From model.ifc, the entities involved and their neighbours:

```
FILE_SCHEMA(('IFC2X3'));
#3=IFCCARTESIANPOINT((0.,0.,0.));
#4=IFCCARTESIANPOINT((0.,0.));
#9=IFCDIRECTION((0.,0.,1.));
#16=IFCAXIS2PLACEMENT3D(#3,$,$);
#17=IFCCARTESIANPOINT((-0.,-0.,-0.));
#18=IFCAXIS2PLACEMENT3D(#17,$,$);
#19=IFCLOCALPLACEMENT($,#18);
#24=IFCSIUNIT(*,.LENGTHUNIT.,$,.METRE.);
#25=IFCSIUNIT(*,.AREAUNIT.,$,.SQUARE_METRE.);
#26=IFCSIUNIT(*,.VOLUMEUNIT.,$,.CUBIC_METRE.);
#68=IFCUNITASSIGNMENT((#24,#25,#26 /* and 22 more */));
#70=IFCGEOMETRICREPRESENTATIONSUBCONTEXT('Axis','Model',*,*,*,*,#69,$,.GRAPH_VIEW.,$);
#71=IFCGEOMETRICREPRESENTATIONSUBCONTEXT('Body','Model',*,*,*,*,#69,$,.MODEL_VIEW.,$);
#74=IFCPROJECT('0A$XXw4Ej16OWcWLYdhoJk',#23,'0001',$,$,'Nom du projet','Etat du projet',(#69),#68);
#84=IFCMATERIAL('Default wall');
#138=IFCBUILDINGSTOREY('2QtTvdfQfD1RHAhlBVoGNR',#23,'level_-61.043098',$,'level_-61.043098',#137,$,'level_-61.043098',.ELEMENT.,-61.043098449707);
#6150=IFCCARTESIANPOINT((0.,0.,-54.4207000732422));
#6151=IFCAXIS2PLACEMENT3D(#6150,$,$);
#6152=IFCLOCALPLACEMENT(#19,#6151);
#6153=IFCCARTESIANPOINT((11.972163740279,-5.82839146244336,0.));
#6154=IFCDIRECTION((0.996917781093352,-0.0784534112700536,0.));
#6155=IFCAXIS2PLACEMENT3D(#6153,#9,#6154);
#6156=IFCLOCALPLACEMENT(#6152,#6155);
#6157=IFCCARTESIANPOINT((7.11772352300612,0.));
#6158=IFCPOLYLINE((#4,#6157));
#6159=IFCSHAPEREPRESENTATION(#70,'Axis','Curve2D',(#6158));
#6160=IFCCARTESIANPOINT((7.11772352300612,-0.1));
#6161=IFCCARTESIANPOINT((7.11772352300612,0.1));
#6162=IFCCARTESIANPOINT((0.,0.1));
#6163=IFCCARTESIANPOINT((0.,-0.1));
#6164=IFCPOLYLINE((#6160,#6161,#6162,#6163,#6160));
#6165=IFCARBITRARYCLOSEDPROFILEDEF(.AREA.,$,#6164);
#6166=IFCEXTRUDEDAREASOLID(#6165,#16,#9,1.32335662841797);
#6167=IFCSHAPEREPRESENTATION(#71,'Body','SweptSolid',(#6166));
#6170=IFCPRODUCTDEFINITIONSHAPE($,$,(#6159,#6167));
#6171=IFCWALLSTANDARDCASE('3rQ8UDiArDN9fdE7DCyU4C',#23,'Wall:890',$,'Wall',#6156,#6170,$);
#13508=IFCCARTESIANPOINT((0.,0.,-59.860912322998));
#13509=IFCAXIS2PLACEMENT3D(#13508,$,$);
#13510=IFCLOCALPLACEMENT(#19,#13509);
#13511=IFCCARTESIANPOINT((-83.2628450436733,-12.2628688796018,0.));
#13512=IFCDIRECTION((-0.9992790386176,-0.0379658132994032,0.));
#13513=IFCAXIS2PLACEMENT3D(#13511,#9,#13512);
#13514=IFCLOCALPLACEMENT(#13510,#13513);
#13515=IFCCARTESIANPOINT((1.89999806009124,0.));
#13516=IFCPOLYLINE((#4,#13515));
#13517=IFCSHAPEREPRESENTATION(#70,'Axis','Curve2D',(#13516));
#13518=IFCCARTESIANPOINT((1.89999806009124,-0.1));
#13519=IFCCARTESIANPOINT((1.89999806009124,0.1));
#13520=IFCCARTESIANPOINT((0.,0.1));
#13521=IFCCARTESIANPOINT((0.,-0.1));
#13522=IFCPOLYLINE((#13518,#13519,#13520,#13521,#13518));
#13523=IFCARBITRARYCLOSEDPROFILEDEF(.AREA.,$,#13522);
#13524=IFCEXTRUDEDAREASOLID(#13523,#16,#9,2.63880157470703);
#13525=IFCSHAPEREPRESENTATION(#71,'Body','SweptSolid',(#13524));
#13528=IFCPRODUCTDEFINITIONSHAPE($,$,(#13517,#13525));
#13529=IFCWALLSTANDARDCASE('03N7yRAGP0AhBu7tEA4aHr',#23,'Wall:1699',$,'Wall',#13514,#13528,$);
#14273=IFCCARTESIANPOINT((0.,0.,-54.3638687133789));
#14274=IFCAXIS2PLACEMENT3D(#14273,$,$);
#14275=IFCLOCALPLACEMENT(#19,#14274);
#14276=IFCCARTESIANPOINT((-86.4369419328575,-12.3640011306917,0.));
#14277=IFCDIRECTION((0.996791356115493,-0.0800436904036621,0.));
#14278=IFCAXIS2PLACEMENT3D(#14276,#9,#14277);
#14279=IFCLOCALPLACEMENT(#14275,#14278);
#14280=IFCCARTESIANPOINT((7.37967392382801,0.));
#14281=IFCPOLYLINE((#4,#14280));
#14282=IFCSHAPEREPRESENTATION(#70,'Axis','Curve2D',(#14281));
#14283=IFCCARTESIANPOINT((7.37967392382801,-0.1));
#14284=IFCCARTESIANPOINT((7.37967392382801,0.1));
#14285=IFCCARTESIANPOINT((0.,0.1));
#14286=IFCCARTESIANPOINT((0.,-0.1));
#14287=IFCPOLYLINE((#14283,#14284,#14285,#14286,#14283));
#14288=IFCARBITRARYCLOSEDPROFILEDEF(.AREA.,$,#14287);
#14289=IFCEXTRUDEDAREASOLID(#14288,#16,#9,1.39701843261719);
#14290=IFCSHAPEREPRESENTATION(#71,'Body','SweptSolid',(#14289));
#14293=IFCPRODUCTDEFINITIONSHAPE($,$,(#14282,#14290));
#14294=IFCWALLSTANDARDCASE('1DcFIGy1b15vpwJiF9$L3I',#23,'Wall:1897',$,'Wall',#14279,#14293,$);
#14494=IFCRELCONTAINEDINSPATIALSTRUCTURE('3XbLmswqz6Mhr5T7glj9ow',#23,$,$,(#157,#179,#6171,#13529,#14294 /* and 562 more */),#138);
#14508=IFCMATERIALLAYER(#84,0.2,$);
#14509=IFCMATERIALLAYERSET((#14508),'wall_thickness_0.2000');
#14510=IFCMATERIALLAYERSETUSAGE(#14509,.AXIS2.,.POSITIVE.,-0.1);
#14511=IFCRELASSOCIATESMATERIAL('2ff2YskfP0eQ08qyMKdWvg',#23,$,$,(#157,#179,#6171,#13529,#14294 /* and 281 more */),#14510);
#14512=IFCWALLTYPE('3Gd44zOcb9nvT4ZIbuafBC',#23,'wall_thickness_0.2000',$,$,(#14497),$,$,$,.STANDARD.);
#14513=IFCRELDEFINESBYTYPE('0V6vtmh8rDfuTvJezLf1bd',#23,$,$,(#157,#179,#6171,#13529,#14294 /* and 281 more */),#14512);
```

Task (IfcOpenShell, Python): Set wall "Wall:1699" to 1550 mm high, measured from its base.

```python
import ifcopenshell
import ifcopenshell.geom
import ifcopenshell.util.representation
import ifcopenshell.util.shape
import ifcopenshell.util.unit

model = ifcopenshell.open("model.ifc")
unit_scale = ifcopenshell.util.unit.calculate_unit_scale(model)
settings = ifcopenshell.geom.settings()


def volume(element):
    """Net volume in cubic metres, openings subtracted."""
    shape = ifcopenshell.geom.create_shape(settings, element)
    return ifcopenshell.util.shape.get_volume(shape.geometry)


wall = model.by_guid("03N7yRAGP0AhBu7tEA4aHr")
before = volume(wall)

body = ifcopenshell.util.representation.get_representation(wall, "Model", "Body")
solid = body.Items[0]
old_height = solid.Depth
solid.Depth = 1.55 / unit_scale
after = volume(wall)

print(f"height {old_height:g} -> {solid.Depth:g}, volume {before:.3f} -> {after:.3f} m3")

model.write("model-out.ifc")
```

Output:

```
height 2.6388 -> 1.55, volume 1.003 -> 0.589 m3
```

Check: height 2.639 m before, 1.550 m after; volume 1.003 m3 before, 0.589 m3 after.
